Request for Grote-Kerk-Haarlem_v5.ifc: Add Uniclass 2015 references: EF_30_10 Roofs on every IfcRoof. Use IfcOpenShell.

First a look at what the model holds.

```python
import ifcopenshell

model = ifcopenshell.open("Grote-Kerk-Haarlem_v5.ifc")
print(model.schema)
print("classifications:", [c.Name for c in model.by_type("IfcClassification")])
for ifc_class in ("IfcDoor", "IfcRoof", "IfcStair", "IfcWall", "IfcWindow"):
    print(ifc_class, len(model.by_type(ifc_class)))
```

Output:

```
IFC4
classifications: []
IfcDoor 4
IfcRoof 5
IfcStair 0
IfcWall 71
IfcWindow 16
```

```python
import ifcopenshell
import ifcopenshell.api.classification

model = ifcopenshell.open("Grote-Kerk-Haarlem_v5.ifc")

system = ifcopenshell.api.classification.add_classification(model, classification="Uniclass 2015")

codes = {
    "IfcRoof": ("EF_30_10", "Roofs"),
}
for ifc_class, (code, name) in codes.items():
    products = model.by_type(ifc_class)
    ifcopenshell.api.classification.add_reference(
        model, products=products, classification=system, identification=code, name=name
    )
    print(code, len(products))

model.write("Grote-Kerk-Haarlem_v5_rev.ifc")
```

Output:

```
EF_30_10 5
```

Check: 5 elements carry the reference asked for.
